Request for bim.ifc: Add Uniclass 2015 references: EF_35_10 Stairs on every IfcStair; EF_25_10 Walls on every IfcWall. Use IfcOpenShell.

First a look at what the model holds.

```python
import ifcopenshell

model = ifcopenshell.open("bim.ifc")
print(model.schema)
print("classifications:", [c.Name for c in model.by_type("IfcClassification")])
for ifc_class in ("IfcDoor", "IfcRoof", "IfcStair", "IfcWall", "IfcWindow"):
    print(ifc_class, len(model.by_type(ifc_class)))
```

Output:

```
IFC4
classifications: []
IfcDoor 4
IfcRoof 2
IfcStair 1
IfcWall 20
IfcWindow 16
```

```python
import ifcopenshell
import ifcopenshell.api.classification

model = ifcopenshell.open("bim.ifc")

system = ifcopenshell.api.classification.add_classification(model, classification="Uniclass 2015")

codes = {
    "IfcStair": ("EF_35_10", "Stairs"),
    "IfcWall": ("EF_25_10", "Walls"),
}
for ifc_class, (code, name) in codes.items():
    products = model.by_type(ifc_class)
    ifcopenshell.api.classification.add_reference(
        model, products=products, classification=system, identification=code, name=name
    )
    print(code, len(products))

model.write("bim_edited.ifc")
```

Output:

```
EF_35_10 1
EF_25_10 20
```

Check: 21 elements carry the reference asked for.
